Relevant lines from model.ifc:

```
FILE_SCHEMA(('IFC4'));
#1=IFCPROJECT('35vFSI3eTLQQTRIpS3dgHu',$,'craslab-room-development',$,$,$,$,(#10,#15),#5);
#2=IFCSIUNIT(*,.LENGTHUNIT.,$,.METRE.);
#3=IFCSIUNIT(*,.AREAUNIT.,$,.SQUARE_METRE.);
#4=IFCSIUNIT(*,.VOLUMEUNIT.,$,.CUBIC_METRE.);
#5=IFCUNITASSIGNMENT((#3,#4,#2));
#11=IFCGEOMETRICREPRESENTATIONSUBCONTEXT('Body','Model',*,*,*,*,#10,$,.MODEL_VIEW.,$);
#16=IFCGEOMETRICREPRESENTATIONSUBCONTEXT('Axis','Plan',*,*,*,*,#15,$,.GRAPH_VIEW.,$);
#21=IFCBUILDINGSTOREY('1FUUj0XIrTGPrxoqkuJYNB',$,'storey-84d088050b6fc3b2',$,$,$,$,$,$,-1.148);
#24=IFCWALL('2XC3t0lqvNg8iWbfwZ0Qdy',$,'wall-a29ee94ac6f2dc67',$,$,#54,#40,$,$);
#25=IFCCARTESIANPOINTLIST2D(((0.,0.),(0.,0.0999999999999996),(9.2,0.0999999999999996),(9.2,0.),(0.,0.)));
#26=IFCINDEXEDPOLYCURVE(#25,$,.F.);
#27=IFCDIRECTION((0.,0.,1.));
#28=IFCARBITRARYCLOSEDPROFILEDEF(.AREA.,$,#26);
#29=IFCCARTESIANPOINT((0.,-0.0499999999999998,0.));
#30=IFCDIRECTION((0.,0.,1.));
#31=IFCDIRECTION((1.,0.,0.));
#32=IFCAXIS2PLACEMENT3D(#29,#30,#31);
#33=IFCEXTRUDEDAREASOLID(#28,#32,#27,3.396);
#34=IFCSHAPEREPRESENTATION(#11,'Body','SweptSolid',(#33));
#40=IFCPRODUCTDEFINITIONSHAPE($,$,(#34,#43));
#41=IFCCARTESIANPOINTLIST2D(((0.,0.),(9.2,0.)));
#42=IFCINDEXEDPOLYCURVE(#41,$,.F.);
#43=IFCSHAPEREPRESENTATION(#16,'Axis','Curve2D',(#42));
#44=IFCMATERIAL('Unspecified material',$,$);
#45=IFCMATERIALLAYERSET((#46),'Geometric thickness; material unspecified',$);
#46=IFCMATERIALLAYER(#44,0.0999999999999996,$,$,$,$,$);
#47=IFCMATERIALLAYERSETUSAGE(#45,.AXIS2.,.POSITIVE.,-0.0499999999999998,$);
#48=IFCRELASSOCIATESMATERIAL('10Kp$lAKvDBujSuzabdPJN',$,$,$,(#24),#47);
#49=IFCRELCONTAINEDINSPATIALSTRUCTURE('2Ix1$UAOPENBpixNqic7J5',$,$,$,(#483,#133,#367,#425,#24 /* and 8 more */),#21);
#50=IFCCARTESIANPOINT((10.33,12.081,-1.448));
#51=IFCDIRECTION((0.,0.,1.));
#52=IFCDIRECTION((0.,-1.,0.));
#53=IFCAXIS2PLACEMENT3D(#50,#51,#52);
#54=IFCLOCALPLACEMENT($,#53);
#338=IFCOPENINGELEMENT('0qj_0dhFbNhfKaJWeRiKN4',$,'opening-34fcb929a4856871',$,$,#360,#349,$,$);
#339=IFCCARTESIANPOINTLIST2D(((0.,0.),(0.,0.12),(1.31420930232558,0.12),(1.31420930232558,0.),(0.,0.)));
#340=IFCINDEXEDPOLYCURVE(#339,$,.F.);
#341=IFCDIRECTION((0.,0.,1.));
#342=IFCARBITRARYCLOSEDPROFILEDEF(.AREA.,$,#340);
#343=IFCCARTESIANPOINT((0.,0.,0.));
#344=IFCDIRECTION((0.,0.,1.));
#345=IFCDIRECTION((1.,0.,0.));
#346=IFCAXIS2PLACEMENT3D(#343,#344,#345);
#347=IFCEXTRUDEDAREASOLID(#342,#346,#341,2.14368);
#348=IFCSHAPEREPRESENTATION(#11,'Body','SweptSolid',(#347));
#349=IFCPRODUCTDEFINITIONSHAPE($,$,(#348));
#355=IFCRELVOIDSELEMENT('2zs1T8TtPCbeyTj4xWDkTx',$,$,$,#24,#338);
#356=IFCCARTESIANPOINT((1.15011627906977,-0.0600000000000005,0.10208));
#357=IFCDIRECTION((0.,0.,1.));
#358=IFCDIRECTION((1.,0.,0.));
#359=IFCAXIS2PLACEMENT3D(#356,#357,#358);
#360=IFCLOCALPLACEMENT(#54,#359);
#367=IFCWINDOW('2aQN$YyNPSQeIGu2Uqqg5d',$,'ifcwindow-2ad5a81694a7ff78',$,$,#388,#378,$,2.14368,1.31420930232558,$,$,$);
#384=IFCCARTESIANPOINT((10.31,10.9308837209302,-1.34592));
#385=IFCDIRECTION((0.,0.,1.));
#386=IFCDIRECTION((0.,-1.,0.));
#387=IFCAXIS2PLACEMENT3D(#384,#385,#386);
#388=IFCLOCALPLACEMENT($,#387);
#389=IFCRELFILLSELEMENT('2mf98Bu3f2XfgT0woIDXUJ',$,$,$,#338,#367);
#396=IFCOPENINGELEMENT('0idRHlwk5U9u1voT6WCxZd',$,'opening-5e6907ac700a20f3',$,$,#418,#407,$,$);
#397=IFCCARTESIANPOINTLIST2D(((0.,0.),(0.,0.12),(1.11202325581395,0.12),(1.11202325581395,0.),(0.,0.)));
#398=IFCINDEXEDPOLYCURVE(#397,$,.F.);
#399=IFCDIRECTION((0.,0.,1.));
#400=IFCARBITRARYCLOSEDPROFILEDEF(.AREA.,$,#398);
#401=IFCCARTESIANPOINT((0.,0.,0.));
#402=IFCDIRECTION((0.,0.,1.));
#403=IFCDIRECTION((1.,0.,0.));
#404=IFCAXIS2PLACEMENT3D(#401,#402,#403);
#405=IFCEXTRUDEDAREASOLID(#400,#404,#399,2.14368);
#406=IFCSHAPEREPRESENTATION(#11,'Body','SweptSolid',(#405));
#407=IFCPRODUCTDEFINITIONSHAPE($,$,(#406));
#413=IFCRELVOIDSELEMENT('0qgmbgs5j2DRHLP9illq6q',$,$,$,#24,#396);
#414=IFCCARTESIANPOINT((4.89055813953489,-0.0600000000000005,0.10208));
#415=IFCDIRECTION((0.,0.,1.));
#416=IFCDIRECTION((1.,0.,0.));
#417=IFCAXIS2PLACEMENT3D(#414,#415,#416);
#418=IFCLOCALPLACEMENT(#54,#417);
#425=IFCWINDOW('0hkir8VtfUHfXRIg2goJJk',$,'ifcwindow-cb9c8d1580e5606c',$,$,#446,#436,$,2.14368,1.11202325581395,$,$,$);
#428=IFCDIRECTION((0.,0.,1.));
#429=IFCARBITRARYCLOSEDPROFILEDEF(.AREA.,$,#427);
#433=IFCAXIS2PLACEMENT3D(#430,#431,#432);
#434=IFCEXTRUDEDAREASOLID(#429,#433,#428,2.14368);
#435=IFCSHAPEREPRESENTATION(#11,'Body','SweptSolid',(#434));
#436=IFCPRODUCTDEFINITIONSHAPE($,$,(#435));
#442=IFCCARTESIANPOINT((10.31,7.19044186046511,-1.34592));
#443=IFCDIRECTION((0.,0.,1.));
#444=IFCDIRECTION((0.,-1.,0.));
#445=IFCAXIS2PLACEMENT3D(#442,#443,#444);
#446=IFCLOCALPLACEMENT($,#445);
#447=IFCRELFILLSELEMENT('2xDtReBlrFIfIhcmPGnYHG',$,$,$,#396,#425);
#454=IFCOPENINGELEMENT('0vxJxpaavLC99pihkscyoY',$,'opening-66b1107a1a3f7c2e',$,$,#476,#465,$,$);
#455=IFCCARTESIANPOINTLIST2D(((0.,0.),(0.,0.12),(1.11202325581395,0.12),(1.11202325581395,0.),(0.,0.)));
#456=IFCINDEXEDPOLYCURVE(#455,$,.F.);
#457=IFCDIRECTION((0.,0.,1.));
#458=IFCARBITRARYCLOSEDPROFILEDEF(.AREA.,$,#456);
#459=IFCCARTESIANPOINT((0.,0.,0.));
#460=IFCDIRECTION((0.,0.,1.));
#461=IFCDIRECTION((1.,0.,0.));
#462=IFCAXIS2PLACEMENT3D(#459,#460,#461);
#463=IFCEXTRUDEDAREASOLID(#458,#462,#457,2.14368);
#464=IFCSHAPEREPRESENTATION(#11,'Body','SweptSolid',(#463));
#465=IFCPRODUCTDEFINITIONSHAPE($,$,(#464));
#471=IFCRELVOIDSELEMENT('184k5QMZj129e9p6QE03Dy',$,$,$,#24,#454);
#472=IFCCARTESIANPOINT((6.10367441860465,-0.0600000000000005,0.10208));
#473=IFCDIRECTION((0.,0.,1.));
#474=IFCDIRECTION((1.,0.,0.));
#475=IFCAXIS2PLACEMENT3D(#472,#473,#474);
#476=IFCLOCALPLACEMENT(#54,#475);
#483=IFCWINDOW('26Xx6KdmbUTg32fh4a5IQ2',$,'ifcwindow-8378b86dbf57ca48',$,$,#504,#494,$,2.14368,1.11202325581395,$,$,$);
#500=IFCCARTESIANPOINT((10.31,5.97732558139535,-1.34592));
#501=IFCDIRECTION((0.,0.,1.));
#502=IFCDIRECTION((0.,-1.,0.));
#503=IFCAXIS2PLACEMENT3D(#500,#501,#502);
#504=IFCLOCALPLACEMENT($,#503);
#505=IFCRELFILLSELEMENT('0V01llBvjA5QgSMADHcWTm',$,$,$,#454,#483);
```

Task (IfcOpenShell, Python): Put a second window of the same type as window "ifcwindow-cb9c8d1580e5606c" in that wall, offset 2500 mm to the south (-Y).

```python
import ifcopenshell
import ifcopenshell.api.feature
import ifcopenshell.api.geometry
import ifcopenshell.api.root
import ifcopenshell.geom
import ifcopenshell.util.element
import ifcopenshell.util.placement
import ifcopenshell.util.shape
import ifcopenshell.util.unit

model = ifcopenshell.open("model.ifc")
unit_scale = ifcopenshell.util.unit.calculate_unit_scale(model)
settings = ifcopenshell.geom.settings()


def volume(element):
    """Net volume in cubic metres, openings subtracted."""
    shape = ifcopenshell.geom.create_shape(settings, element)
    return ifcopenshell.util.shape.get_volume(shape.geometry)


window = model.by_guid("0hkir8VtfUHfXRIg2goJJk")
opening = window.FillsVoids[0].RelatingOpeningElement
wall = opening.VoidsElements[0].RelatingBuildingElement
before = volume(wall)
shift = ifcopenshell.util.placement.get_local_placement(wall.ObjectPlacement)[:3, 0] * 2.5 / unit_scale

# copy_class copies the void relationship, type, container and properties, but no geometry.
new_opening = ifcopenshell.api.root.copy_class(model, product=opening)
new_opening.Representation = ifcopenshell.util.element.copy_deep(
    model, opening.Representation, exclude=["IfcGeometricRepresentationContext", "IfcRepresentationMap"]
)
new_window = ifcopenshell.api.root.copy_class(model, product=window)
new_window.Representation = ifcopenshell.util.element.copy_deep(
    model, window.Representation, exclude=["IfcGeometricRepresentationContext", "IfcRepresentationMap"]
)
ifcopenshell.api.feature.add_filling(model, opening=new_opening, element=new_window)

for old, new in ((opening, new_opening), (window, new_window)):
    matrix = ifcopenshell.util.placement.get_local_placement(old.ObjectPlacement)
    matrix[:3, 3] += shift
    ifcopenshell.api.geometry.edit_object_placement(model, product=new, matrix=matrix, is_si=False)

after = volume(wall)

print(f"wall volume {before:.3f} -> {after:.3f} m3")

model.write("model_v2.ifc")
```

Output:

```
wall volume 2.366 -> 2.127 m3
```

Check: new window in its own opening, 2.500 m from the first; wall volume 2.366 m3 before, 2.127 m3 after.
